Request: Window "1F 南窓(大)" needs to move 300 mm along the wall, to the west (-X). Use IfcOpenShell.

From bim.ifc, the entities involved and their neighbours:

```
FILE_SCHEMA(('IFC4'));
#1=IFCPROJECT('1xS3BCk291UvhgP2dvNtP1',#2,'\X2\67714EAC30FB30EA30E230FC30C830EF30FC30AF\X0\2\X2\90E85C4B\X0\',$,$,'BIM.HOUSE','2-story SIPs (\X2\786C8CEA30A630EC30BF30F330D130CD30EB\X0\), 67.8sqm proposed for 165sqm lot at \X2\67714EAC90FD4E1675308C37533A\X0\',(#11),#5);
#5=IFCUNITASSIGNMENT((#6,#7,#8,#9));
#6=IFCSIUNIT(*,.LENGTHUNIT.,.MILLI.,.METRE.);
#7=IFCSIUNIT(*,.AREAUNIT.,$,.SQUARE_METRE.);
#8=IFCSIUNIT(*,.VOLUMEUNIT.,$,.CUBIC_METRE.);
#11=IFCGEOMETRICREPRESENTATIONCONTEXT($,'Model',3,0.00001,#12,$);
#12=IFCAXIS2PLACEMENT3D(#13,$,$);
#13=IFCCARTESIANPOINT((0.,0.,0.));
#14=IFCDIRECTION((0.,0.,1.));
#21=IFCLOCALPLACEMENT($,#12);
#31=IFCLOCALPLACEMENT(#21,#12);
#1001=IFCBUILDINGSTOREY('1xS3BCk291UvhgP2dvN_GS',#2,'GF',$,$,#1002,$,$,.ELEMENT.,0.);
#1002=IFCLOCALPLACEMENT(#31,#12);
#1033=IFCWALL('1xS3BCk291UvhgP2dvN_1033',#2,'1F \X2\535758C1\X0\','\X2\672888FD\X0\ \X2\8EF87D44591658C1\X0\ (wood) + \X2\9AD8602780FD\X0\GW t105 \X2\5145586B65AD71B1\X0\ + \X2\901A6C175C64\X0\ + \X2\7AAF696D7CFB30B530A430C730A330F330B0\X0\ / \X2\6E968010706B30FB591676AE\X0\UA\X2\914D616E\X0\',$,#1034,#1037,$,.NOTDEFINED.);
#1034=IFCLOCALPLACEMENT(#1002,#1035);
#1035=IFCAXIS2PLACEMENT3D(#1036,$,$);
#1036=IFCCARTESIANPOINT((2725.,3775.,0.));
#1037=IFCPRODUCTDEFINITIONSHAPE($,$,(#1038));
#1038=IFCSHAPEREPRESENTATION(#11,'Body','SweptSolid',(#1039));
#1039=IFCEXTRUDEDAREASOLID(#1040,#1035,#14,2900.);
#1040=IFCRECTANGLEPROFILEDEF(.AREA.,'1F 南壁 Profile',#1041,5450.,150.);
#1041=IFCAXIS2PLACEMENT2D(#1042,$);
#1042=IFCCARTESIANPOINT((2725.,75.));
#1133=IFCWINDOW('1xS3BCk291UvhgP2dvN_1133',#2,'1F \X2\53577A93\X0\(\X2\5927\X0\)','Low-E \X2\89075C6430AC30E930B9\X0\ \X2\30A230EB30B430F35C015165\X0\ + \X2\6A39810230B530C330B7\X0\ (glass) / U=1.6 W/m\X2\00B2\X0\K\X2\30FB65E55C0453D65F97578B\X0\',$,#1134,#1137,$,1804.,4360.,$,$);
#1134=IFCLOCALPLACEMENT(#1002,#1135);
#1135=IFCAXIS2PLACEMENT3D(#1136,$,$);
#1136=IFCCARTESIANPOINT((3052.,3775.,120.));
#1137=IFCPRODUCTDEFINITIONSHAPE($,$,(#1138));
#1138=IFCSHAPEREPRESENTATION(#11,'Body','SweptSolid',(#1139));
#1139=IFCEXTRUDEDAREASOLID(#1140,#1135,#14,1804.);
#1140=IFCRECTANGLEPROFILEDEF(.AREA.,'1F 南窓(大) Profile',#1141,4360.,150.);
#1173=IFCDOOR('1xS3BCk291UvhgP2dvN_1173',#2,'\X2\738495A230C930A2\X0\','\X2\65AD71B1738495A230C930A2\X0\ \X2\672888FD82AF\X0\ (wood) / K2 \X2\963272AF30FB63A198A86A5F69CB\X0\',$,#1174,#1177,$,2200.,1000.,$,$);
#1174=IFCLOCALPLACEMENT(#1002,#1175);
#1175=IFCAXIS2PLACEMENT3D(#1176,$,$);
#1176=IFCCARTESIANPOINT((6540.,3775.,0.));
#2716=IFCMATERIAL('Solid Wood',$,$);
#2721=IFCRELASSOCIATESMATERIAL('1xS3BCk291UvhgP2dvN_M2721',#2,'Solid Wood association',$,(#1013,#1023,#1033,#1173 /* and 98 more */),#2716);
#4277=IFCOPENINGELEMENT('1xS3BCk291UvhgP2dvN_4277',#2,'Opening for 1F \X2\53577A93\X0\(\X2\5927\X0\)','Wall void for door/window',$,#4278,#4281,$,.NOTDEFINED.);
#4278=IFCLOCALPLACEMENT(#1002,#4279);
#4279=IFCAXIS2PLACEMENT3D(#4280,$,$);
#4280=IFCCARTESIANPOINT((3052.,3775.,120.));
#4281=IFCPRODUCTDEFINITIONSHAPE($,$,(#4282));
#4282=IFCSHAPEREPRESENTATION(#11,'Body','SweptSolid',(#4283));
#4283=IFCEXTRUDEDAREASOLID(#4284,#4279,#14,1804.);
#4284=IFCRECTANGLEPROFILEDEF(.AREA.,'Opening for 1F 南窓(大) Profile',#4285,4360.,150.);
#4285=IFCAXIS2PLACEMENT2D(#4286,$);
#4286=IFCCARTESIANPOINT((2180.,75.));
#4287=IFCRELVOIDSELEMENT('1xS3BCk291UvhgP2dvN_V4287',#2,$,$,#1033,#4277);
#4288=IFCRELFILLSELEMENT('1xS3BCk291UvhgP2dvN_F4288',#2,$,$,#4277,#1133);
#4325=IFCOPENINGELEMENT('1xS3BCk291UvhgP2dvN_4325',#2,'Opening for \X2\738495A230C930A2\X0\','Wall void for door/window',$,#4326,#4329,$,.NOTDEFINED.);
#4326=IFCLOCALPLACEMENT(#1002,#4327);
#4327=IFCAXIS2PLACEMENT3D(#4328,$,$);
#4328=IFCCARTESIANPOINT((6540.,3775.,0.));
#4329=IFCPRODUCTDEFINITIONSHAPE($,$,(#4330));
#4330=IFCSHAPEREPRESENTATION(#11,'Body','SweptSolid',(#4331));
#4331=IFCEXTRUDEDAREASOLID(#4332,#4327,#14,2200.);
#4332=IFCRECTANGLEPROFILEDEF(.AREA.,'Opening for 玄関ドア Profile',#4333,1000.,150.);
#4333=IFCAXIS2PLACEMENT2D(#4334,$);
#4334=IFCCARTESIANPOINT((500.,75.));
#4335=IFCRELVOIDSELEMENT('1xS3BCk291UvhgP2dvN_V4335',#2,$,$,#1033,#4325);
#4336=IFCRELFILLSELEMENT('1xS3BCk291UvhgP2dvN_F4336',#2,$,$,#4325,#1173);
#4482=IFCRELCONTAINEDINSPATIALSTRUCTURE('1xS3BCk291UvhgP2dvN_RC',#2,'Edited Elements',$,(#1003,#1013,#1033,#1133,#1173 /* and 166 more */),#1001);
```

```python
import ifcopenshell
import ifcopenshell.api.geometry
import ifcopenshell.util.placement

model = ifcopenshell.open("bim.ifc")

window = model.by_guid("1xS3BCk291UvhgP2dvN_1133")
opening = window.FillsVoids[0].RelatingOpeningElement
wall = opening.VoidsElements[0].RelatingBuildingElement

wall_matrix = ifcopenshell.util.placement.get_local_placement(wall.ObjectPlacement)
shift = wall_matrix[:3, 0] * -300.0
before = ifcopenshell.util.placement.get_local_placement(window.ObjectPlacement)[:3, 3].copy()

# The window is not placed relative to its opening, so move both.
for product in (opening, window):
    matrix = ifcopenshell.util.placement.get_local_placement(product.ObjectPlacement)
    matrix[:3, 3] += shift
    ifcopenshell.api.geometry.edit_object_placement(model, product=product, matrix=matrix, is_si=False)

after = ifcopenshell.util.placement.get_local_placement(window.ObjectPlacement)[:3, 3]
print("window moved by", (after - before).round(3) + 0.0)

model.write("bim_v2.ifc")
```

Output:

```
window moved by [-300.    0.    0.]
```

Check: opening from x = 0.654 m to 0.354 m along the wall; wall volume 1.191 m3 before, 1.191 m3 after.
